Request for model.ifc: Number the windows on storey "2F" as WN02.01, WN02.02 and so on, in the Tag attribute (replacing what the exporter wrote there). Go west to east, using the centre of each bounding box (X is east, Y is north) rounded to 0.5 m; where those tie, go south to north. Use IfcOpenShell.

First a look at what the model holds.

```python
import ifcopenshell
import ifcopenshell.util.element
import ifcopenshell.util.placement

model = ifcopenshell.open("model.ifc")
print(model.schema)
storey = next(s for s in model.by_type("IfcBuildingStorey") if s.Name == "2F")
windows = [e for e in ifcopenshell.util.element.get_decomposition(storey) if e.is_a("IfcWindow")]
for e in sorted(windows, key=lambda e: e.id()):
    origin = ifcopenshell.util.placement.get_local_placement(e.ObjectPlacement)[:3, 3]
    print(e.id(), e.Tag, e.Name, origin.round(2) + 0.0, sep=" | ")
```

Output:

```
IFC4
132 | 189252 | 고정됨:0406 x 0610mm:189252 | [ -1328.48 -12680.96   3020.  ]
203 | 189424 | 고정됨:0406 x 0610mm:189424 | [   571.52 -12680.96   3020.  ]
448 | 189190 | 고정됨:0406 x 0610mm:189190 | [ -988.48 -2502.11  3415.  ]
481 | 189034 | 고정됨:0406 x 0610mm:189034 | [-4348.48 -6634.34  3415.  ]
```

```python
import ifcopenshell
import ifcopenshell.geom
import ifcopenshell.util.element
import ifcopenshell.util.shape

model = ifcopenshell.open("model.ifc")
settings = ifcopenshell.geom.settings()
settings.set("use-world-coords", True)


def centre(element):
    shape = ifcopenshell.geom.create_shape(settings, element)
    return ifcopenshell.util.shape.get_bbox_centroid(shape.geometry)


storey = next(s for s in model.by_type("IfcBuildingStorey") if s.Name == "2F")
windows = [e for e in ifcopenshell.util.element.get_decomposition(storey) if e.is_a("IfcWindow")]

# Insertion points can sit at a corner or the storey origin, so sort by the geometry (in metres).
centres = {e: centre(e) for e in windows}
windows.sort(key=lambda e: (round(centres[e][0] / 0.5), centres[e][1]))

for i, e in enumerate(windows, start=1):
    number = f"WN02.{i:02d}"
    e.Tag = number
    print(e.id(), number)

model.write("model-out.ifc")
```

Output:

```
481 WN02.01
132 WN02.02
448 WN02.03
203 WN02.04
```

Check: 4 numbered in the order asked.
